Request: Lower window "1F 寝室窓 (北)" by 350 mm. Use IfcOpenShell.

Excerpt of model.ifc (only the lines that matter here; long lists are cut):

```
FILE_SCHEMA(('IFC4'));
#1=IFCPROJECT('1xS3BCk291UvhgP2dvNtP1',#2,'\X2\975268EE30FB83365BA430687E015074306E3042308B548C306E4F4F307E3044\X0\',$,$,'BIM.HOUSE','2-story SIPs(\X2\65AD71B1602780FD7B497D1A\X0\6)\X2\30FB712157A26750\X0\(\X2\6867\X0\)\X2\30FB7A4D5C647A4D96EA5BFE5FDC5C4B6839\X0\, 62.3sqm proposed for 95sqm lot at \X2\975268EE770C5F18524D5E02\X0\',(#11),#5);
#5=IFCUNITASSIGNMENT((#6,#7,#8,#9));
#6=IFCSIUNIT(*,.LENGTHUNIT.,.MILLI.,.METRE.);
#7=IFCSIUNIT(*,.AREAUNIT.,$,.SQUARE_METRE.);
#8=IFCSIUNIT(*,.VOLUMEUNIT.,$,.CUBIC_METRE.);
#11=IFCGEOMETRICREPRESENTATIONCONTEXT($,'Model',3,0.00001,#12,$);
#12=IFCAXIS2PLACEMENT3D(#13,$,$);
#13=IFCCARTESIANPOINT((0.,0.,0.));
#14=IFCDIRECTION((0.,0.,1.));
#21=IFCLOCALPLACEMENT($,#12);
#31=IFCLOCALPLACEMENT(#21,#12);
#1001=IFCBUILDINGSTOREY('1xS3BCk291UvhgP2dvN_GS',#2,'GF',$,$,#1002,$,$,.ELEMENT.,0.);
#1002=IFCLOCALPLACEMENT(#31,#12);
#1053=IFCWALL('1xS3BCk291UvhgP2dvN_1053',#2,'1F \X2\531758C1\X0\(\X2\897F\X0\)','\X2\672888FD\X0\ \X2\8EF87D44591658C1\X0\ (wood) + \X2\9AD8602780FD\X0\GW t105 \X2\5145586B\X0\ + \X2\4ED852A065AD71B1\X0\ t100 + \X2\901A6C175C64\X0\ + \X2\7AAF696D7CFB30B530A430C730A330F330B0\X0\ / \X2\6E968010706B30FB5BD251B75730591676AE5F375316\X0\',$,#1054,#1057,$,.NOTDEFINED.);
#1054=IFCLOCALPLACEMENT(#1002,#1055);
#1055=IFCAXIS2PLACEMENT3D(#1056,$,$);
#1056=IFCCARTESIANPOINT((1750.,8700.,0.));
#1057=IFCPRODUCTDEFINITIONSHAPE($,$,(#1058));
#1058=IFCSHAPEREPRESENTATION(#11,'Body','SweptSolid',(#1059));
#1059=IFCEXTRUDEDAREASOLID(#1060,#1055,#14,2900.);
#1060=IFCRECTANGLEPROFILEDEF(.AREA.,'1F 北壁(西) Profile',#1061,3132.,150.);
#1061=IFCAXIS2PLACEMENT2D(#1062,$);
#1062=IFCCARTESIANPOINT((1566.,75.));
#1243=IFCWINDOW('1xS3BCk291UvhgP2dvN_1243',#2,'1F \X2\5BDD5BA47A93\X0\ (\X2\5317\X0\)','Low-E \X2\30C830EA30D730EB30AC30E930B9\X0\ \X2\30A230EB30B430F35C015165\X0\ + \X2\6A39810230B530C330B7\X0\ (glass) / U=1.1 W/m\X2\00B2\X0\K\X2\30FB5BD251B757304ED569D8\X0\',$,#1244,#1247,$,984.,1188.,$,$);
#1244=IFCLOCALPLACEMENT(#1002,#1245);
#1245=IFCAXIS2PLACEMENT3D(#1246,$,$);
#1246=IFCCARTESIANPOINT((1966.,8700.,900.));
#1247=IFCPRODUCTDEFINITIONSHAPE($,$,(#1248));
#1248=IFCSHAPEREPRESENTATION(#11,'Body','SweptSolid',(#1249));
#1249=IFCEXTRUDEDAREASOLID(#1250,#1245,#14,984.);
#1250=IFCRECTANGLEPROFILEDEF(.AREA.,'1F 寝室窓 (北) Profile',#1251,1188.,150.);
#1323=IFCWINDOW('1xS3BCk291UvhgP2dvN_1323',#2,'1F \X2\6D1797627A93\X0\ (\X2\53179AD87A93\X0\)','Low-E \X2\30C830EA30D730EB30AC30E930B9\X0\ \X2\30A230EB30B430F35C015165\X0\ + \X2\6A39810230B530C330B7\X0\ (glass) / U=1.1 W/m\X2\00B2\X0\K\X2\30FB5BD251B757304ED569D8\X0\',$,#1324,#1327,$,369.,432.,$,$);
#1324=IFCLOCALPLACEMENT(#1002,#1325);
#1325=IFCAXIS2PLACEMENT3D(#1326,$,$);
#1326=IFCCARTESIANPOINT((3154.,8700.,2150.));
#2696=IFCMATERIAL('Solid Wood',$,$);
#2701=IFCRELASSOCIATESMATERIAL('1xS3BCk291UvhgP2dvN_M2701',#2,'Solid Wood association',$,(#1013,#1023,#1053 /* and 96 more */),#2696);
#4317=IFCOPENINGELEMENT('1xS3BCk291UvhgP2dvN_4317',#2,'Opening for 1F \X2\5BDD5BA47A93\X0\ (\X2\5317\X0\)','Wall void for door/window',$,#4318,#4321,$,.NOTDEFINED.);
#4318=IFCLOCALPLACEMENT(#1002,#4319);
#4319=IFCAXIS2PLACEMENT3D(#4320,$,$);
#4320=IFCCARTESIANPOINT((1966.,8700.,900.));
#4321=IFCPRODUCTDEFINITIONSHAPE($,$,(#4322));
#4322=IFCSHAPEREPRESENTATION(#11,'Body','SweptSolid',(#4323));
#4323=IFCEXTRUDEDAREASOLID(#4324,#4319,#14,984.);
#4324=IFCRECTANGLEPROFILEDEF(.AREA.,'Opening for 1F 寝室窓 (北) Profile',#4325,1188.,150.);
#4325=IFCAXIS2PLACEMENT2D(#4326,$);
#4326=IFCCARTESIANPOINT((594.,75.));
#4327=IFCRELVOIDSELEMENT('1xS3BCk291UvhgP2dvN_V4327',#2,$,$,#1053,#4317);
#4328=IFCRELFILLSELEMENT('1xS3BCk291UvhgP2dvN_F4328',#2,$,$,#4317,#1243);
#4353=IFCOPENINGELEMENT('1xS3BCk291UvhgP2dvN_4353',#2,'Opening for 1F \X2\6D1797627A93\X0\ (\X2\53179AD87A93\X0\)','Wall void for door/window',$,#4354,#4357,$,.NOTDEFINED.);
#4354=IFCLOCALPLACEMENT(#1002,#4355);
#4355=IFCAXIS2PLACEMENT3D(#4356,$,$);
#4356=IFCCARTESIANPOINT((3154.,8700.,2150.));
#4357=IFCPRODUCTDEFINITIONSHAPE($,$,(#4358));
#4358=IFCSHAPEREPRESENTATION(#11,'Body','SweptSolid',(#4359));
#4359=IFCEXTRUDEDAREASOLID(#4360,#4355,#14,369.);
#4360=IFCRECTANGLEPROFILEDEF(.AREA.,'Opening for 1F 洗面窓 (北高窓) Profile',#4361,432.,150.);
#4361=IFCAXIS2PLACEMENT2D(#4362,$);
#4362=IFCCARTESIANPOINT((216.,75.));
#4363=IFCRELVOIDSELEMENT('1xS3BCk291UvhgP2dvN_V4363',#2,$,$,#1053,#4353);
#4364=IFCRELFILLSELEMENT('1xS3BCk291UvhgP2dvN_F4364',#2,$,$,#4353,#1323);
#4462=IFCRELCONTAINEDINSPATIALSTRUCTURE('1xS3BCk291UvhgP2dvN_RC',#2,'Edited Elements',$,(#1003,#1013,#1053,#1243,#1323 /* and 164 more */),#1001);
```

```python
import numpy as np
import ifcopenshell
import ifcopenshell.api.geometry
import ifcopenshell.util.placement
import ifcopenshell.util.unit

model = ifcopenshell.open("model.ifc")
unit_scale = ifcopenshell.util.unit.calculate_unit_scale(model)

window = model.by_id(1243)
opening = window.FillsVoids[0].RelatingOpeningElement
dz = -350.0

shift = np.array([0.0, 0.0, dz])
# The window is not placed relative to its opening, so move both.
for product in (opening, window):
    matrix = ifcopenshell.util.placement.get_local_placement(product.ObjectPlacement)
    matrix[:3, 3] += shift
    ifcopenshell.api.geometry.edit_object_placement(model, product=product, matrix=matrix, is_si=False)

print(f"moved by {dz * unit_scale:+.3f} m")

model.write("model_updated.ifc")
```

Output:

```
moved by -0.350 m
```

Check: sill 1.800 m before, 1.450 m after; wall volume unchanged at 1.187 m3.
